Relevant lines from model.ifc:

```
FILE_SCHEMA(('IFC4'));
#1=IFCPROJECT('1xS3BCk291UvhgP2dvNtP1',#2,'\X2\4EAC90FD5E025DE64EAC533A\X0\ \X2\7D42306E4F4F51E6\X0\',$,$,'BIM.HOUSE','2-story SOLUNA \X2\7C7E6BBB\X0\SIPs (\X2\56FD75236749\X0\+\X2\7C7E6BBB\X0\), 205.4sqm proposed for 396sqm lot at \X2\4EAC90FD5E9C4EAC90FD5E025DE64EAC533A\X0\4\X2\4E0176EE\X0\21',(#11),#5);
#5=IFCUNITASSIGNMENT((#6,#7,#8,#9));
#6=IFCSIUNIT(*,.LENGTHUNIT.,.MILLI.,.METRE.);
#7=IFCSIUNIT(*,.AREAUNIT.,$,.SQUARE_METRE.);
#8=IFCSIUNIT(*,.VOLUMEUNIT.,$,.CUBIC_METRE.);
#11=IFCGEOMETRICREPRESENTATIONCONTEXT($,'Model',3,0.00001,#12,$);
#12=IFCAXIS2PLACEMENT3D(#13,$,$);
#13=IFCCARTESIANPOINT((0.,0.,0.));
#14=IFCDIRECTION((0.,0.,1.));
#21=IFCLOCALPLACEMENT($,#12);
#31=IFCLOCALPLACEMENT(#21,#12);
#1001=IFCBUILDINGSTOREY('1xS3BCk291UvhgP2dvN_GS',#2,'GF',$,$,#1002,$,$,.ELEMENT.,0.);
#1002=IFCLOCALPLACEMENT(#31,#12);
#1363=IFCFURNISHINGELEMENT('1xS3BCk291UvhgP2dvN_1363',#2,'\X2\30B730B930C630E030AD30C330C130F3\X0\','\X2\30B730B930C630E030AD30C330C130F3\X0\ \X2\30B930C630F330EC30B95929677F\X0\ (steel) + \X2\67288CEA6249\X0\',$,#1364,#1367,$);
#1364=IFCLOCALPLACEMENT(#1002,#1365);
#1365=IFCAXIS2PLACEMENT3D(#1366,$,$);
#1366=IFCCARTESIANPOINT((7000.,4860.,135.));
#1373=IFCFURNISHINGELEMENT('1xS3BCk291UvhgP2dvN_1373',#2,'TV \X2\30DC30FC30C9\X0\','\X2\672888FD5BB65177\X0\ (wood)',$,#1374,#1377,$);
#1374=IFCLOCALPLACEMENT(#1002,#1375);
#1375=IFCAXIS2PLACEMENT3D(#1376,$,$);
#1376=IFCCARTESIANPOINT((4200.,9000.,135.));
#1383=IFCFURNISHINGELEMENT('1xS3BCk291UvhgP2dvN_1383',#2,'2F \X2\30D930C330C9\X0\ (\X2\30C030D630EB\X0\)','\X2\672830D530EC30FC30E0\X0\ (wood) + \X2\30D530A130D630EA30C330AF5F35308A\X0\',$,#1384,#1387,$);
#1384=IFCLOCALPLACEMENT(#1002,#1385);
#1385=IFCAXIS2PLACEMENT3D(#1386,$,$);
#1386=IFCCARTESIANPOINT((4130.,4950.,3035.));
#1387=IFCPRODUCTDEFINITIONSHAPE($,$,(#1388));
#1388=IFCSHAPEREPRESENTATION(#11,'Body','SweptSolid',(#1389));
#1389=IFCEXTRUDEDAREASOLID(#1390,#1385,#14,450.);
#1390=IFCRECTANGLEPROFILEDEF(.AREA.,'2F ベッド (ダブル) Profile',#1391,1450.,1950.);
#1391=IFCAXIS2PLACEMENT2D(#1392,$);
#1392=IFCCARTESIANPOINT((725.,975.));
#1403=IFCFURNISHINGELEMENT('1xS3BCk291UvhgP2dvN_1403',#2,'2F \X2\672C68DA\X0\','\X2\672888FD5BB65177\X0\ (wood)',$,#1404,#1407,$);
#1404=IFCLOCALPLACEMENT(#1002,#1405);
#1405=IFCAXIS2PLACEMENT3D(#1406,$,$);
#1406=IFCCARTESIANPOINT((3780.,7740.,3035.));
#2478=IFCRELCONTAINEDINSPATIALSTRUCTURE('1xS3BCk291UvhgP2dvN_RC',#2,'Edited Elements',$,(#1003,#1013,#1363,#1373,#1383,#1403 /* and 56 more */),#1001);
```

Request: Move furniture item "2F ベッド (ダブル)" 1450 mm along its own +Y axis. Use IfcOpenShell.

```python
import ifcopenshell
import ifcopenshell.api.geometry
import ifcopenshell.util.placement

model = ifcopenshell.open("model.ifc")

item = model.by_guid("1xS3BCk291UvhgP2dvN_1383")
matrix = ifcopenshell.util.placement.get_local_placement(item.ObjectPlacement)
matrix[:3, 3] += matrix[:3, 1] * 1450.0
ifcopenshell.api.geometry.edit_object_placement(model, product=item, matrix=matrix, is_si=False)

print(ifcopenshell.util.placement.get_local_placement(item.ObjectPlacement).round(3) + 0.0)

model.write("model_edited.ifc")
```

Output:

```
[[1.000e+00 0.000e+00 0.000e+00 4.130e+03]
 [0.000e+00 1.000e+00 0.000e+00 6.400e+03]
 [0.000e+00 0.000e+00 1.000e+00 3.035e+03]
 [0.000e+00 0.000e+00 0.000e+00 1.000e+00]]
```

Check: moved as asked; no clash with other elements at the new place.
